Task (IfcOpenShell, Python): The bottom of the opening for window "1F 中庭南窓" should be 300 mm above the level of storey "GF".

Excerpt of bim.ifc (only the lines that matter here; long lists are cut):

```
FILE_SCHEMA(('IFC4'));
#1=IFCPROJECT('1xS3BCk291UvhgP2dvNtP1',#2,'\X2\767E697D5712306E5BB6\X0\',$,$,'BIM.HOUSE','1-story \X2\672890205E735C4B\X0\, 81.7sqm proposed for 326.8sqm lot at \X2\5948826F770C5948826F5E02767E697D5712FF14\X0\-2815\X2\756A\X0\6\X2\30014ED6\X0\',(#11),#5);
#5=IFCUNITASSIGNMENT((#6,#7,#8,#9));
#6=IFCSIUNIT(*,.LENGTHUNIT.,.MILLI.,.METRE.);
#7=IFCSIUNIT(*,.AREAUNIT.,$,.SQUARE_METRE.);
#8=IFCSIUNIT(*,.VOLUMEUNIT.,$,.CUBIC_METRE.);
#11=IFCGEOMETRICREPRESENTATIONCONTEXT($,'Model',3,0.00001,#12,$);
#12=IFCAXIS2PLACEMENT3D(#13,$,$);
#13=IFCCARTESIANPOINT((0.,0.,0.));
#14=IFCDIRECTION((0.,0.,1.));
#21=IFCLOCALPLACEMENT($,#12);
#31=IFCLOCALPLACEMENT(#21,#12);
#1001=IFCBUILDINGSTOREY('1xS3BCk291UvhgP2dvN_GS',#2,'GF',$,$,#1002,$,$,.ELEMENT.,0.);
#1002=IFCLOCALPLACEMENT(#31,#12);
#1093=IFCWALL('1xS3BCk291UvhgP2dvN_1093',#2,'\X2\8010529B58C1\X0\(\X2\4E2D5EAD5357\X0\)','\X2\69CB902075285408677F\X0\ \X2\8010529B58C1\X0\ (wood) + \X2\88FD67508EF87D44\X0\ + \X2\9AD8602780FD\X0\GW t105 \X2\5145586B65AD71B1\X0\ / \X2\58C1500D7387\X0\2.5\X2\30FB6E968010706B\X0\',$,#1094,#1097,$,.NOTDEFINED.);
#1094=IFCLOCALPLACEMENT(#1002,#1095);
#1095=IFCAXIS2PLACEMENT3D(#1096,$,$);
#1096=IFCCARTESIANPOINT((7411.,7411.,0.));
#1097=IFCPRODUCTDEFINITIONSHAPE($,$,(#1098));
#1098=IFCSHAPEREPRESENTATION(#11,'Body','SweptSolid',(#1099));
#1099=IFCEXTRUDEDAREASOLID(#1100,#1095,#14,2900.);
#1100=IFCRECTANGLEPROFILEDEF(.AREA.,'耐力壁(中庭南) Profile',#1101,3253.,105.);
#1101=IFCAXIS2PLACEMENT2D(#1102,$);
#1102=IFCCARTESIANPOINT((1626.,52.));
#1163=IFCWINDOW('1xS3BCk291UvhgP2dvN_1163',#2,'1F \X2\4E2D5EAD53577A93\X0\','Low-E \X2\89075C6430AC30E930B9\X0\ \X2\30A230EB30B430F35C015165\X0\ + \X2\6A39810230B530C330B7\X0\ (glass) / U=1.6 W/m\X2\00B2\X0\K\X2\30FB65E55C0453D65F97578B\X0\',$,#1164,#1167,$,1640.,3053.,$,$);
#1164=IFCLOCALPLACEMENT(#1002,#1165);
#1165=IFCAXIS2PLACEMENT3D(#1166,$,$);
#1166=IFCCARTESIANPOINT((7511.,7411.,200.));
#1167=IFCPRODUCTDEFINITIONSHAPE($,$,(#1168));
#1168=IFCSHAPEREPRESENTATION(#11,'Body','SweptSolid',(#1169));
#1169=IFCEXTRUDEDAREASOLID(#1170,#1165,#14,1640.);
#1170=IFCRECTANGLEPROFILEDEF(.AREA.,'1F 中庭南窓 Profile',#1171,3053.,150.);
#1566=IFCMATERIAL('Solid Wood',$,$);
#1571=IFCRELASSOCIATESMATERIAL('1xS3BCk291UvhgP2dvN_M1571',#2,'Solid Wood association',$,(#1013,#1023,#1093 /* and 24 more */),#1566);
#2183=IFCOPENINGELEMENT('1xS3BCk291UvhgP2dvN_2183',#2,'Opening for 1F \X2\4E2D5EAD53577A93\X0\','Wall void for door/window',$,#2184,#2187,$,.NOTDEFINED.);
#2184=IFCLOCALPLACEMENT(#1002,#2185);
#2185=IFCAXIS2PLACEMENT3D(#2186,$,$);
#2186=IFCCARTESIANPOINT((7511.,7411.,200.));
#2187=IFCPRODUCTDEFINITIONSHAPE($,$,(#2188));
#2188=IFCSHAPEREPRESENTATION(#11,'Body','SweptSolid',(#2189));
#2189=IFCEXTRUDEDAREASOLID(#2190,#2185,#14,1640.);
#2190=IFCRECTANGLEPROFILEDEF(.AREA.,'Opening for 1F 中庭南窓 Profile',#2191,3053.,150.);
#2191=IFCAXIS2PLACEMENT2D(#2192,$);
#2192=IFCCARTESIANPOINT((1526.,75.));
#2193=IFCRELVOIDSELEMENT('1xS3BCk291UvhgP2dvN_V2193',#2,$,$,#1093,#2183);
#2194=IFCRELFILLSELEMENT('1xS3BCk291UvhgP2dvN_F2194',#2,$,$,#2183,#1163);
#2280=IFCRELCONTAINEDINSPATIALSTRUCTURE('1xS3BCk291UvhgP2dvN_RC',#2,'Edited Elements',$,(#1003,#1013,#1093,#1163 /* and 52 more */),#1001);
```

```python
import numpy as np
import ifcopenshell
import ifcopenshell.api.geometry
import ifcopenshell.geom
import ifcopenshell.util.element
import ifcopenshell.util.placement
import ifcopenshell.util.shape
import ifcopenshell.util.unit

model = ifcopenshell.open("bim.ifc")
unit_scale = ifcopenshell.util.unit.calculate_unit_scale(model)

window = model.by_guid("1xS3BCk291UvhgP2dvN_1163")
opening = window.FillsVoids[0].RelatingOpeningElement
storey = ifcopenshell.util.element.get_container(window, ifc_class="IfcBuildingStorey")
level = ifcopenshell.util.placement.get_local_placement(storey.ObjectPlacement)[2, 3]

# The opening's origin need not be at the sill, so measure its lowest point.
shape = ifcopenshell.geom.create_shape(ifcopenshell.geom.settings(), opening)
bottom = ifcopenshell.util.shape.get_shape_bottom_elevation(shape, shape.geometry) / unit_scale
dz = level + 300.0 - bottom

shift = np.array([0.0, 0.0, dz])
# The window is not placed relative to its opening, so move both.
for product in (opening, window):
    matrix = ifcopenshell.util.placement.get_local_placement(product.ObjectPlacement)
    matrix[:3, 3] += shift
    ifcopenshell.api.geometry.edit_object_placement(model, product=product, matrix=matrix, is_si=False)

print(f"moved by {dz * unit_scale:+.3f} m")

model.write("bim_rev.ifc")
```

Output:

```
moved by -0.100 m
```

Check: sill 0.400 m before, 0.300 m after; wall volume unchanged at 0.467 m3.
